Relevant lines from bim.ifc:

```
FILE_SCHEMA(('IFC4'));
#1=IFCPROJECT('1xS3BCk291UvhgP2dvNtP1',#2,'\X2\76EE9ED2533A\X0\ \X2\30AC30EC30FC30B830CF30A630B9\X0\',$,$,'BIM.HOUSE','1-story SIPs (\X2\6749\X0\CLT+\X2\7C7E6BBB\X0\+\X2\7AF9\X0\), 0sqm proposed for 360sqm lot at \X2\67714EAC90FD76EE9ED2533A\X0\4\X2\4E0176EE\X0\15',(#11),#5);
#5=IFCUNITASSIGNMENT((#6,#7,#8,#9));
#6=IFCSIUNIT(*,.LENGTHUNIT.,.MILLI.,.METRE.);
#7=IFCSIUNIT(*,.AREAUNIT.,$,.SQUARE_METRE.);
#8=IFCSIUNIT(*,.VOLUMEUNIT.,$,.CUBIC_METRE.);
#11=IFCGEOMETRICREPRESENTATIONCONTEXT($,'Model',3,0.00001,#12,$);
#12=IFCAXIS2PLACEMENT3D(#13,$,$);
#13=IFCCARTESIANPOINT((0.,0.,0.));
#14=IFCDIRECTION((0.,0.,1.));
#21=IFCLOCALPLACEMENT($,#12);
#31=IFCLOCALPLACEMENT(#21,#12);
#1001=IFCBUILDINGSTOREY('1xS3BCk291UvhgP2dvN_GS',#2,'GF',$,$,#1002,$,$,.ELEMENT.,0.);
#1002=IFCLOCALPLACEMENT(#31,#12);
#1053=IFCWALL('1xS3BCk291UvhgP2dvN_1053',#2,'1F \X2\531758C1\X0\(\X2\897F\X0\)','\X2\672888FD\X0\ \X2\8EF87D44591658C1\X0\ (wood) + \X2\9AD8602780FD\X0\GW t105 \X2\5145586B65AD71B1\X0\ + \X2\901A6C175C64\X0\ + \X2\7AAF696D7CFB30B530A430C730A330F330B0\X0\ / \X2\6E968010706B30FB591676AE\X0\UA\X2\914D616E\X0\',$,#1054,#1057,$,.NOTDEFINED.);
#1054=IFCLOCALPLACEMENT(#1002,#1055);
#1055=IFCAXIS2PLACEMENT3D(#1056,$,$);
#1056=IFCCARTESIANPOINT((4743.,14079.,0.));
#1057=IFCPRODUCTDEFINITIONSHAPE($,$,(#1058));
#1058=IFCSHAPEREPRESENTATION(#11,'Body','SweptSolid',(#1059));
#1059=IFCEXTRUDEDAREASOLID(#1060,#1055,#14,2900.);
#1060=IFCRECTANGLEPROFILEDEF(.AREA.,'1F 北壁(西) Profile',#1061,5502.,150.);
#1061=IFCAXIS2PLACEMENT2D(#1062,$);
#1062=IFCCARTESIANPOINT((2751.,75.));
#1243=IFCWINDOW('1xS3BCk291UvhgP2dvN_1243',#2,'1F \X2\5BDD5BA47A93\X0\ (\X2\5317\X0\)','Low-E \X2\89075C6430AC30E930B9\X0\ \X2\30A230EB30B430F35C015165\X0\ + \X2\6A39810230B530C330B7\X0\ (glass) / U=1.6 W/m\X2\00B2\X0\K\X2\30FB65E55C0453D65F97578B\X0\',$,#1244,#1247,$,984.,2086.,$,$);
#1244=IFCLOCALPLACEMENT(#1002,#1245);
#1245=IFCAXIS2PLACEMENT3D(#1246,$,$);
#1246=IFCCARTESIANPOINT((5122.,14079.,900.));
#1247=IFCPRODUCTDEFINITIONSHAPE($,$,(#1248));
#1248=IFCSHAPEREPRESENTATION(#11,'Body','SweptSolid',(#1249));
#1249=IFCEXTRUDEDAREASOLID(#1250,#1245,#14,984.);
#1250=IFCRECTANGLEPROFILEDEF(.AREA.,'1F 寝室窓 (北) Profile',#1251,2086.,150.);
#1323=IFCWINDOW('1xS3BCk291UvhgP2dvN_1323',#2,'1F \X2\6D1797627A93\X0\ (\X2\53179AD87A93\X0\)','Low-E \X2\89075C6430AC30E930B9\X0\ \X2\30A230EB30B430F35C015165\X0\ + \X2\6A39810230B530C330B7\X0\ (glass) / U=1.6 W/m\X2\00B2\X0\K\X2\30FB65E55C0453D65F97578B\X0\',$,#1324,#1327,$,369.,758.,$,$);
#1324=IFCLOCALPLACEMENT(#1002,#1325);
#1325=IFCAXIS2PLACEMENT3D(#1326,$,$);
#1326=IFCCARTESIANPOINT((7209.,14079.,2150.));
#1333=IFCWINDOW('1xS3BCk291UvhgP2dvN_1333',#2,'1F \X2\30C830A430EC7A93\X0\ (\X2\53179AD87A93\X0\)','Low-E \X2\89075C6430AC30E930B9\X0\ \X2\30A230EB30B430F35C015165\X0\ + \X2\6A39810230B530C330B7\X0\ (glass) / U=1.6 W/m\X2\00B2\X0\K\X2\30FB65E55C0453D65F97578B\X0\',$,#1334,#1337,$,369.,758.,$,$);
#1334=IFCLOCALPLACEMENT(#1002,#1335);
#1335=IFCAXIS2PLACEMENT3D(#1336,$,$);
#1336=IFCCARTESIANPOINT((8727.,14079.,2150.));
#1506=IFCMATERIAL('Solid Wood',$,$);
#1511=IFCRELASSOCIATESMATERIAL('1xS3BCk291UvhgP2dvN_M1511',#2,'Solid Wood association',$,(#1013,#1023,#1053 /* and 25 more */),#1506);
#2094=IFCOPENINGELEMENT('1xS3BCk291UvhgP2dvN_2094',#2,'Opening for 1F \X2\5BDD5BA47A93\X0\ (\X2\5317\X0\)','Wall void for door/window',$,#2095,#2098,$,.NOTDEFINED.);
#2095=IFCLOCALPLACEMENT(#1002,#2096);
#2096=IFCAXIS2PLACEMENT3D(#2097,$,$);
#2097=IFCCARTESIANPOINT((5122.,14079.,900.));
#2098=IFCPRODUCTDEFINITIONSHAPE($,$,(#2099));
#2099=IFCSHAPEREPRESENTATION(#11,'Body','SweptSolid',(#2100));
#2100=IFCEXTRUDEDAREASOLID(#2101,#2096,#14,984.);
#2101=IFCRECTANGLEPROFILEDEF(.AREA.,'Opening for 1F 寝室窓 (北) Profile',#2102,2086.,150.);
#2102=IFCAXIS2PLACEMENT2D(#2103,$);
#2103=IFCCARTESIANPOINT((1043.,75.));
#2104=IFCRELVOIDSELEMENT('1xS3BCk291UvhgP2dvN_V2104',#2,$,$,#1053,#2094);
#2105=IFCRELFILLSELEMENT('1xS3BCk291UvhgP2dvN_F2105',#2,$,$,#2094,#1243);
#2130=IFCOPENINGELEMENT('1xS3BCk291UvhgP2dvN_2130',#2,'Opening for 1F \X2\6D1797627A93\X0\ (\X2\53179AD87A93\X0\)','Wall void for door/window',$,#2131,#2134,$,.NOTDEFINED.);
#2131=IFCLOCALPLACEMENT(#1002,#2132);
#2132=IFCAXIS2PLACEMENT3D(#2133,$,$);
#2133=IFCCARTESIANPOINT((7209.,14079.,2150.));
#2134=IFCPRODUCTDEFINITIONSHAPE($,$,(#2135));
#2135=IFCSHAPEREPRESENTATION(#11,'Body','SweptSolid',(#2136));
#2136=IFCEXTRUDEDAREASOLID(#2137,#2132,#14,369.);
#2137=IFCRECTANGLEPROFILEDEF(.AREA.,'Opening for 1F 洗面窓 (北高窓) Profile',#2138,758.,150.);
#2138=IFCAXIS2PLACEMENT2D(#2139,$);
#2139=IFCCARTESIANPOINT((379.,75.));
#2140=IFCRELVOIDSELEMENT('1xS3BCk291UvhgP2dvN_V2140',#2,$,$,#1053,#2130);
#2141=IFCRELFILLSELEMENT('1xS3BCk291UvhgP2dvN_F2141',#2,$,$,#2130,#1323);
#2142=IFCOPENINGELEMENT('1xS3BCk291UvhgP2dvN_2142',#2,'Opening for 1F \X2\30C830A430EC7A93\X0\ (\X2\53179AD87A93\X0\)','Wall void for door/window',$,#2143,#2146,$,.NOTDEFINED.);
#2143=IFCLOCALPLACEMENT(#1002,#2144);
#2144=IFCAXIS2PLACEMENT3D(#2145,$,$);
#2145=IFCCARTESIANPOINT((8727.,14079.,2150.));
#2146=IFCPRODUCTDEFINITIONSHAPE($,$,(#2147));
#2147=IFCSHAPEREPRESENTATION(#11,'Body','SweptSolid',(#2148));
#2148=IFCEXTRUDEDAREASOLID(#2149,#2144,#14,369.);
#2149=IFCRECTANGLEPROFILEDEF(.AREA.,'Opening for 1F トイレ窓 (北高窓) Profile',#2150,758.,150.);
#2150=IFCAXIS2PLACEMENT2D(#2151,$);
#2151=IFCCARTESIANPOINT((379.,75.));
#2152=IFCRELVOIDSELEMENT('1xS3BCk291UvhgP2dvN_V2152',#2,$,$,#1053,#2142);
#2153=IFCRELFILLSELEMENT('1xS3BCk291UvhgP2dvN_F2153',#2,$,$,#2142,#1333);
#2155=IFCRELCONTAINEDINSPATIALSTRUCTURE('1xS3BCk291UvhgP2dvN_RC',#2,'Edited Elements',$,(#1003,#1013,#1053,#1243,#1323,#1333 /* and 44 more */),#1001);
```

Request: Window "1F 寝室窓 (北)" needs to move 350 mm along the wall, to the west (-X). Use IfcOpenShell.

```python
import ifcopenshell
import ifcopenshell.api.geometry
import ifcopenshell.util.placement

model = ifcopenshell.open("bim.ifc")

window = model.by_id(1243)
opening = window.FillsVoids[0].RelatingOpeningElement
wall = opening.VoidsElements[0].RelatingBuildingElement

wall_matrix = ifcopenshell.util.placement.get_local_placement(wall.ObjectPlacement)
shift = wall_matrix[:3, 0] * -350.0
before = ifcopenshell.util.placement.get_local_placement(window.ObjectPlacement)[:3, 3].copy()

# The window is not placed relative to its opening, so move both.
for product in (opening, window):
    matrix = ifcopenshell.util.placement.get_local_placement(product.ObjectPlacement)
    matrix[:3, 3] += shift
    ifcopenshell.api.geometry.edit_object_placement(model, product=product, matrix=matrix, is_si=False)

after = ifcopenshell.util.placement.get_local_placement(window.ObjectPlacement)[:3, 3]
print("window moved by", (after - before).round(3) + 0.0)

model.write("bim_rev.ifc")
```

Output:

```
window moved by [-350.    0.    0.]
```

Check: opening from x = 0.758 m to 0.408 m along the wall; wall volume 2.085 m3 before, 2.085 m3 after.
